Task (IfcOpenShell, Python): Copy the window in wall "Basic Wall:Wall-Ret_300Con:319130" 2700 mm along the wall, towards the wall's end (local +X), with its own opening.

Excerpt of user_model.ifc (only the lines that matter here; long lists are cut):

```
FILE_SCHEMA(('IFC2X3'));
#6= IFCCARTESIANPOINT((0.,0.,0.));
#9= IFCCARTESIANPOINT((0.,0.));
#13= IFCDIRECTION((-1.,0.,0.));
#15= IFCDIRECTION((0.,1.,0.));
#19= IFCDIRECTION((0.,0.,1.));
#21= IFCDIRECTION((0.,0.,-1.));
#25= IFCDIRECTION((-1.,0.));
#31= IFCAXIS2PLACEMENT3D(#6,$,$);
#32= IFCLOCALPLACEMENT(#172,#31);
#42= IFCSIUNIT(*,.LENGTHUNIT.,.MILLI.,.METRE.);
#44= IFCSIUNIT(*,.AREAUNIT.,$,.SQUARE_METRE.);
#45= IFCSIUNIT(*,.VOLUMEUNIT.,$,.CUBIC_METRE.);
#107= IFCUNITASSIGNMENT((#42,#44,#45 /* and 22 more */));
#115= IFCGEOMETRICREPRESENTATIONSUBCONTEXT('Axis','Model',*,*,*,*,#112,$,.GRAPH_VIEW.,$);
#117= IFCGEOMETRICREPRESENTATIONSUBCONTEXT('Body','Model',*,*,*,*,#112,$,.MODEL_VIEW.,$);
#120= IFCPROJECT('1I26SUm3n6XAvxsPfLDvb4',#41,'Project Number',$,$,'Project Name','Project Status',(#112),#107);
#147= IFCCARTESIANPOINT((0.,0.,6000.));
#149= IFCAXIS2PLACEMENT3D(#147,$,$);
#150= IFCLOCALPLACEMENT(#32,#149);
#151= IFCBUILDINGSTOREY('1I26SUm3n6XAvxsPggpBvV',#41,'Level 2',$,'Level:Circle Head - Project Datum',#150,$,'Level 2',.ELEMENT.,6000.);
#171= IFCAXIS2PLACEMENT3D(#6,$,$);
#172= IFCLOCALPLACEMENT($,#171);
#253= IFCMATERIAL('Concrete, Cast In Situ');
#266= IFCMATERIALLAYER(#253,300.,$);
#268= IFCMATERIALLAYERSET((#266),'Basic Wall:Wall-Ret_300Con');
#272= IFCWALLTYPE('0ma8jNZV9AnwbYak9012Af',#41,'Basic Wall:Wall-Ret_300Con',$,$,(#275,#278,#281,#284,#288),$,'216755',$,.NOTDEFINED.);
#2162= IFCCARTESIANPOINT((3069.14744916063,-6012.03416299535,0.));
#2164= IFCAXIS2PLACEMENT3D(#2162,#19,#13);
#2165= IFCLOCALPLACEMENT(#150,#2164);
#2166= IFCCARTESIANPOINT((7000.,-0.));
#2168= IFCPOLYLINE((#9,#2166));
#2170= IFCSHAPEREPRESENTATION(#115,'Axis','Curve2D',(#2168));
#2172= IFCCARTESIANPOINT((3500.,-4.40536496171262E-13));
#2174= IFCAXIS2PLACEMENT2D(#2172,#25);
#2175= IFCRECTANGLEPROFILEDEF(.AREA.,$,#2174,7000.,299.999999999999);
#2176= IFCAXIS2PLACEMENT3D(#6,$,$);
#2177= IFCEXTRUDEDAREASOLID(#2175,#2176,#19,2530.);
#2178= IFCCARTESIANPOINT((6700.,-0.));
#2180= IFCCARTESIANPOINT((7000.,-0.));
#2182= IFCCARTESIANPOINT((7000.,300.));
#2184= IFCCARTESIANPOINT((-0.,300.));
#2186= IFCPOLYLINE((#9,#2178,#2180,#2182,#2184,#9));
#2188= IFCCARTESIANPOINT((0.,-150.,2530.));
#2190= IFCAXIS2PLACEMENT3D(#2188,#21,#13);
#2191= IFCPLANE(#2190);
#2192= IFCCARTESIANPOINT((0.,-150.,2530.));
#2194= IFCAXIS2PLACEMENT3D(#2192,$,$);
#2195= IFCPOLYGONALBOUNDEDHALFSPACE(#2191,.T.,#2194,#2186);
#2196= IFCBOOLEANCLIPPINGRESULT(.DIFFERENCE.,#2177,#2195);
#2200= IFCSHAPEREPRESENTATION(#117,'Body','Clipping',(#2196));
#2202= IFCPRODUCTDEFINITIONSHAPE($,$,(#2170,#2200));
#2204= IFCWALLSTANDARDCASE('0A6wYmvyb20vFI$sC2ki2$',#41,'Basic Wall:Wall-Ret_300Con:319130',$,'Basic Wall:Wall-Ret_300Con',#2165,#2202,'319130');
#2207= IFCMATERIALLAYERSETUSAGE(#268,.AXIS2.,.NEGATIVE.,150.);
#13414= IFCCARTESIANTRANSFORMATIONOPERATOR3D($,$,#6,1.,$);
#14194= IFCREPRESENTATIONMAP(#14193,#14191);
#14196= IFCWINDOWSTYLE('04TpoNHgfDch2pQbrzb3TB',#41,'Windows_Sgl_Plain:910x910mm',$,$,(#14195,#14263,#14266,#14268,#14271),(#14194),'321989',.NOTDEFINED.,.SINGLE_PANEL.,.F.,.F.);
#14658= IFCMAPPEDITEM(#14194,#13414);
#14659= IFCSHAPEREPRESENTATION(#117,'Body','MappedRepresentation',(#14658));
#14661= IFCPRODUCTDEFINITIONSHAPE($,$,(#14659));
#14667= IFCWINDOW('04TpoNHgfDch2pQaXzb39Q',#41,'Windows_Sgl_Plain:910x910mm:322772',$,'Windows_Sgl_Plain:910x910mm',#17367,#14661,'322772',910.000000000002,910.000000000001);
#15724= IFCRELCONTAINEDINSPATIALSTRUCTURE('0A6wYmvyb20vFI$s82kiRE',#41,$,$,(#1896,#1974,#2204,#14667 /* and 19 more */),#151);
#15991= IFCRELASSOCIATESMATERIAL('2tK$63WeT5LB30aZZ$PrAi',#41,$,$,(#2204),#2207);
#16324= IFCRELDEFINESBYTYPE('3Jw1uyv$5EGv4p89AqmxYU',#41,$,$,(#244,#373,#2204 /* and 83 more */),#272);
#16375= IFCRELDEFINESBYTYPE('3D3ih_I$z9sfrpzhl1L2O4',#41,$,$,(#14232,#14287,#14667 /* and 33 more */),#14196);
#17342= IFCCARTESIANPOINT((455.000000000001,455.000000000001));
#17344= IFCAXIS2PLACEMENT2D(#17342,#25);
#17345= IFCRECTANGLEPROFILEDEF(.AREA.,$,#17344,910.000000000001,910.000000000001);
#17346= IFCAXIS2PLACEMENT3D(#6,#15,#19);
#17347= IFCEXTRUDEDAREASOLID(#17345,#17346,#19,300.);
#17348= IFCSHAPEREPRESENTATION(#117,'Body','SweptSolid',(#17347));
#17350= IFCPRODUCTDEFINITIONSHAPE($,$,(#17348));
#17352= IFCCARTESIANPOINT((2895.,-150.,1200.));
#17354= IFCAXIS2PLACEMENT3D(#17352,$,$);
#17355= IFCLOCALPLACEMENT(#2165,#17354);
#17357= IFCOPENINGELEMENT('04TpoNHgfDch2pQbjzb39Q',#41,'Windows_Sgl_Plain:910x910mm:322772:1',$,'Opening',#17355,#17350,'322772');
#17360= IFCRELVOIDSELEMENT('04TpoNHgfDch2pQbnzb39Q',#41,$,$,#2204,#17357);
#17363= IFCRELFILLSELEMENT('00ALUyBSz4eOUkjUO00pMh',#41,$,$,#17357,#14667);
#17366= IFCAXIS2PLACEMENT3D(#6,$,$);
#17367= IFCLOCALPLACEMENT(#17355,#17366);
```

```python
import ifcopenshell
import ifcopenshell.api.feature
import ifcopenshell.api.geometry
import ifcopenshell.api.root
import ifcopenshell.geom
import ifcopenshell.util.element
import ifcopenshell.util.placement
import ifcopenshell.util.shape

model = ifcopenshell.open("user_model.ifc")
settings = ifcopenshell.geom.settings()


def volume(element):
    """Net volume in cubic metres, openings subtracted."""
    shape = ifcopenshell.geom.create_shape(settings, element)
    return ifcopenshell.util.shape.get_volume(shape.geometry)


def reuse_history(source, copy):
    """copy_class also copies each property set's owner history, people and application; keep the originals."""
    for rel in copy.IsDefinedBy:
        if rel.is_a("IfcRelDefinesByProperties") and (history := rel.RelatingPropertyDefinition.OwnerHistory):
            rel.RelatingPropertyDefinition.OwnerHistory = source.OwnerHistory
            ifcopenshell.util.element.remove_deep2(model, history)


window = model.by_id(14667)
opening = window.FillsVoids[0].RelatingOpeningElement
wall = opening.VoidsElements[0].RelatingBuildingElement
before = volume(wall)
shift = ifcopenshell.util.placement.get_local_placement(wall.ObjectPlacement)[:3, 0] * 2700.0

# copy_class copies the void relationship, type, container and properties, but no geometry.
new_opening = ifcopenshell.api.root.copy_class(model, product=opening)
new_opening.Representation = ifcopenshell.util.element.copy_deep(
    model, opening.Representation, exclude=["IfcGeometricRepresentationContext", "IfcRepresentationMap"]
)
new_opening.Name = "Windows_Sgl_Plain:910x910mm"
new_opening.Tag = None
new_window = ifcopenshell.api.root.copy_class(model, product=window)
new_window.Representation = ifcopenshell.util.element.copy_deep(
    model, window.Representation, exclude=["IfcGeometricRepresentationContext", "IfcRepresentationMap"]
)
new_window.Name = "Windows_Sgl_Plain:910x910mm"
new_window.Tag = None
reuse_history(window, new_window)
fills = ifcopenshell.api.feature.add_filling(model, opening=new_opening, element=new_window)
fills.OwnerHistory = new_window.OwnerHistory  # required in IFC2X3

for old, new in ((opening, new_opening), (window, new_window)):
    matrix = ifcopenshell.util.placement.get_local_placement(old.ObjectPlacement)
    matrix[:3, 3] += shift
    ifcopenshell.api.geometry.edit_object_placement(model, product=new, matrix=matrix, is_si=False)

after = volume(wall)

print(f"wall volume {before:.3f} -> {after:.3f} m3")

model.write("user_model_rev.ifc")
```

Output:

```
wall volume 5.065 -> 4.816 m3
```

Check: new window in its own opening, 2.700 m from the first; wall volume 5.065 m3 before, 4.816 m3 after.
